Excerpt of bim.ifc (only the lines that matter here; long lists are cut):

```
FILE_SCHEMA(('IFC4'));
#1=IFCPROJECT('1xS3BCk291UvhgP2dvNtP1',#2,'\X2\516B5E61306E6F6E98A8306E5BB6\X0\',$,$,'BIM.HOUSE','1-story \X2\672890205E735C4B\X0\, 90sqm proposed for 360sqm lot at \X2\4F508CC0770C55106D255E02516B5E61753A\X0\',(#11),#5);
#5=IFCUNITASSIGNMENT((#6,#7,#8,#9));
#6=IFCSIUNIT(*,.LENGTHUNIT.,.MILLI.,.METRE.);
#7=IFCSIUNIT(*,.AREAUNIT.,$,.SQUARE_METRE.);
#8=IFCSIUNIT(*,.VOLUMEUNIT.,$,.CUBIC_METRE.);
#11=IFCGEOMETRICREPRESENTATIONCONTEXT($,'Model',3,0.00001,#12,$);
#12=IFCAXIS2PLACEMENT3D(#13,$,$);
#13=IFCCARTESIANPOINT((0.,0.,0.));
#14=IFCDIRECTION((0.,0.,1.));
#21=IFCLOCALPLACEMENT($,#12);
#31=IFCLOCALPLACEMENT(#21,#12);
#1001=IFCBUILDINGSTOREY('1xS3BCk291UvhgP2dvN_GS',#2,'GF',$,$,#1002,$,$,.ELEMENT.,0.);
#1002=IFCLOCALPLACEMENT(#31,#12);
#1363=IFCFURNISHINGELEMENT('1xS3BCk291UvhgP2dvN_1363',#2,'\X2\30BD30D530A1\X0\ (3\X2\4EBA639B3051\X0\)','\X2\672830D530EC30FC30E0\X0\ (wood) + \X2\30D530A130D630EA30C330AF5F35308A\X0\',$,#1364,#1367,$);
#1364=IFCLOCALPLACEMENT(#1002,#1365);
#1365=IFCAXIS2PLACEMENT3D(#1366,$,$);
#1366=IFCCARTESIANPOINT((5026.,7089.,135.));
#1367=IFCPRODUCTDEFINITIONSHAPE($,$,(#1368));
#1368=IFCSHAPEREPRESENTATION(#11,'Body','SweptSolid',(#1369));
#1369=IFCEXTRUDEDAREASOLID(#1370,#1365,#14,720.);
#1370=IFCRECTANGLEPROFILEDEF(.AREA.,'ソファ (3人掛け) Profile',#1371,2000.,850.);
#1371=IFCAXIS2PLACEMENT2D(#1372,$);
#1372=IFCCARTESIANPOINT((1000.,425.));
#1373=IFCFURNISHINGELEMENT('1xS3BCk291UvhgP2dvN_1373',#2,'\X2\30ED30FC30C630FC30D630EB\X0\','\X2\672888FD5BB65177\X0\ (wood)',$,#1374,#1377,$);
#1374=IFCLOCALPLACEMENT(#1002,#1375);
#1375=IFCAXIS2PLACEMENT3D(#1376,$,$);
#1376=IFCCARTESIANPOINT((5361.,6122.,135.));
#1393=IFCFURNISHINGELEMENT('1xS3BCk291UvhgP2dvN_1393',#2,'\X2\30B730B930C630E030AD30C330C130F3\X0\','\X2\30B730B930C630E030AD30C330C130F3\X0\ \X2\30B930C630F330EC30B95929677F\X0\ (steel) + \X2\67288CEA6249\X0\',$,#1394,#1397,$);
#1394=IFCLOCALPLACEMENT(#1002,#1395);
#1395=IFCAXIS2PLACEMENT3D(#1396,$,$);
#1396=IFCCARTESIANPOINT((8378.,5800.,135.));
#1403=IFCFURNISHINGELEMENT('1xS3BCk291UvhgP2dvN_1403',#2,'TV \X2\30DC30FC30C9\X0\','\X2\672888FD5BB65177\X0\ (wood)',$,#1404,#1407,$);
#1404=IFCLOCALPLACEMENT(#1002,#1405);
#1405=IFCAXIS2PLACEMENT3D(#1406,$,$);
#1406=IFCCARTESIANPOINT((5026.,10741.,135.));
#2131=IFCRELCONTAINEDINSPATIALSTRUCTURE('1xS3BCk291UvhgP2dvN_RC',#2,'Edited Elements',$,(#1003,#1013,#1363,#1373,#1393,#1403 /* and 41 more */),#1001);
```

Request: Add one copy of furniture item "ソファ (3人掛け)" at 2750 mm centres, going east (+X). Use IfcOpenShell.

```python
import numpy as np
import ifcopenshell
import ifcopenshell.api.geometry
import ifcopenshell.api.root
import ifcopenshell.util.element
import ifcopenshell.util.placement
import ifcopenshell.util.unit

model = ifcopenshell.open("bim.ifc")
unit_scale = ifcopenshell.util.unit.calculate_unit_scale(model)


def reuse_history(source, copy):
    """copy_class also copies each property set's owner history, people and application; keep the originals."""
    for rel in copy.IsDefinedBy:
        if rel.is_a("IfcRelDefinesByProperties") and (history := rel.RelatingPropertyDefinition.OwnerHistory):
            rel.RelatingPropertyDefinition.OwnerHistory = source.OwnerHistory
            ifcopenshell.util.element.remove_deep2(model, history)


source = model.by_guid("1xS3BCk291UvhgP2dvN_1363")
base = ifcopenshell.util.placement.get_local_placement(source.ObjectPlacement)
step = np.array([1.0, 0.0, 0.0]) * 2.75 / unit_scale

for i in range(1, 2):
    copy = ifcopenshell.api.root.copy_class(model, product=source)
    copy.Representation = ifcopenshell.util.element.copy_deep(
        model, source.Representation, exclude=["IfcGeometricRepresentationContext", "IfcRepresentationMap"]
    )
    reuse_history(source, copy)
    matrix = base.copy()
    matrix[:3, 3] += i * step
    print("added at", matrix[:3, 3].round(3) + 0.0)
    ifcopenshell.api.geometry.edit_object_placement(model, product=copy, matrix=matrix, is_si=False)

model.write("bim-out.ifc")
```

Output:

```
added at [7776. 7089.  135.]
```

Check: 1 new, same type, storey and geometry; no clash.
